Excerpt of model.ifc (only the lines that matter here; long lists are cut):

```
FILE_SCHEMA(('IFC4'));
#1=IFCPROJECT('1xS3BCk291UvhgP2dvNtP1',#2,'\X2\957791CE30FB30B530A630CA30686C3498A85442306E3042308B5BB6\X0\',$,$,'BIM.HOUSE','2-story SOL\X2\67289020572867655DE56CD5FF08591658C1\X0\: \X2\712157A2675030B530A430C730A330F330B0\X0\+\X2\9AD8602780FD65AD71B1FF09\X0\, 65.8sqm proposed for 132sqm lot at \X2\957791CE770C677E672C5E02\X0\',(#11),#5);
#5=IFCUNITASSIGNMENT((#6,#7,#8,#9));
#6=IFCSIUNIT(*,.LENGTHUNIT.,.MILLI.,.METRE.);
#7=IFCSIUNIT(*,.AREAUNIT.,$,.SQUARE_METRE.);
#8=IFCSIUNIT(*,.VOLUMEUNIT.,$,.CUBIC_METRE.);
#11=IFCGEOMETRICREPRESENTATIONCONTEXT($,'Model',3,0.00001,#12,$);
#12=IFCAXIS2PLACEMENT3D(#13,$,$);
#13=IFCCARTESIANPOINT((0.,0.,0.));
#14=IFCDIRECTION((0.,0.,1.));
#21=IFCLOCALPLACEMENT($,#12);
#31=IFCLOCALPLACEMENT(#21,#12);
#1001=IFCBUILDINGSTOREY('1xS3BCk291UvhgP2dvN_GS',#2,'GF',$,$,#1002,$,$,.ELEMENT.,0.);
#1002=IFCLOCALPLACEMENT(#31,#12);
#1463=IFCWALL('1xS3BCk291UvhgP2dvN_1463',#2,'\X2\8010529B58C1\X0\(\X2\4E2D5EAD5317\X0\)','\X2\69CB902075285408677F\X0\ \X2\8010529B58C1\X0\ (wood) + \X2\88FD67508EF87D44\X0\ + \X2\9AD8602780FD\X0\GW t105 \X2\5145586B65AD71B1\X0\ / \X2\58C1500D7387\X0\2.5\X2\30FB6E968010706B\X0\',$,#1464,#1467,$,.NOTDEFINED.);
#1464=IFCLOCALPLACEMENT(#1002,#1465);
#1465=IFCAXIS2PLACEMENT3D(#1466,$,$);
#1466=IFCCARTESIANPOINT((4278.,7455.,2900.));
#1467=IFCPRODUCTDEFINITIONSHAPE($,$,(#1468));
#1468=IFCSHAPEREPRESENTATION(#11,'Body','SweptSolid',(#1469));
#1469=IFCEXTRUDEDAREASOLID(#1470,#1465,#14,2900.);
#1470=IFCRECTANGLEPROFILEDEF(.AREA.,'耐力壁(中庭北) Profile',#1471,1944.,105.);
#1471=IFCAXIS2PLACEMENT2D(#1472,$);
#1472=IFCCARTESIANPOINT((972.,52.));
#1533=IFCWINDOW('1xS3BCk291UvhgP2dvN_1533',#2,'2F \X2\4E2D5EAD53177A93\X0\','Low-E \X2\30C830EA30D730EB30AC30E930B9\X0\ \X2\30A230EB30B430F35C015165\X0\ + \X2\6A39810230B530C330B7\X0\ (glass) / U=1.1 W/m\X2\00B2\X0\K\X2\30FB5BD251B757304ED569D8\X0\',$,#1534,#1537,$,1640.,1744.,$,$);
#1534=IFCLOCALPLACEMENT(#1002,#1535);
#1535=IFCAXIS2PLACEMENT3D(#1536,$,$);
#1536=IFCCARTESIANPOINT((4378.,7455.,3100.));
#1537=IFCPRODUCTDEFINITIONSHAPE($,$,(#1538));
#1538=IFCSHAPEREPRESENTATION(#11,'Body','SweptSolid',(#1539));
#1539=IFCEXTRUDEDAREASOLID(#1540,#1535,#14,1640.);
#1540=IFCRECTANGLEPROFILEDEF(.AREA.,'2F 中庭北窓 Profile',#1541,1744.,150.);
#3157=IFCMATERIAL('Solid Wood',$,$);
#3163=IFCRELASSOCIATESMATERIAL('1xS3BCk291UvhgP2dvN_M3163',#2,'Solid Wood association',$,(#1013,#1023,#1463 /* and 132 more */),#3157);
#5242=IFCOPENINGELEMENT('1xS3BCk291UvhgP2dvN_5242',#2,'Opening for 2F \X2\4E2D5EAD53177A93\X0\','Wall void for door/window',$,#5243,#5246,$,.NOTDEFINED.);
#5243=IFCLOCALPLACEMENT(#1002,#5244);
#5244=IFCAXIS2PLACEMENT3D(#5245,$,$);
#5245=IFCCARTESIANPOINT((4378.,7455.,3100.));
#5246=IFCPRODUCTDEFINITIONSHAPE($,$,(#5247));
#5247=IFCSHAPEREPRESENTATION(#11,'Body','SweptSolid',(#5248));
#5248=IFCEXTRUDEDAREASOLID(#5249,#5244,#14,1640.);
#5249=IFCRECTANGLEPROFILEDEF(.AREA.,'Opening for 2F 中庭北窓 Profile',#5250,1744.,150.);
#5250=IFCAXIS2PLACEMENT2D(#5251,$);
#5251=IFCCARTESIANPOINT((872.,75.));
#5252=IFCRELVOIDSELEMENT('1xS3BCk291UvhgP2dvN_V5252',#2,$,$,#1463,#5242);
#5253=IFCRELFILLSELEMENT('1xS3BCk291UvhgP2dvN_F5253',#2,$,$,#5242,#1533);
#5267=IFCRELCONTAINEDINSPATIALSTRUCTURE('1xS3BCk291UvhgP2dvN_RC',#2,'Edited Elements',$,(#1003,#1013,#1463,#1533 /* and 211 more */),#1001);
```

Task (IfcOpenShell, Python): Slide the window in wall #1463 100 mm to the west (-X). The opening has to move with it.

```python
import ifcopenshell
import ifcopenshell.api.geometry
import ifcopenshell.util.placement
import ifcopenshell.util.unit

model = ifcopenshell.open("model.ifc")
unit_scale = ifcopenshell.util.unit.calculate_unit_scale(model)

window = model.by_guid("1xS3BCk291UvhgP2dvN_1533")
opening = window.FillsVoids[0].RelatingOpeningElement
wall = opening.VoidsElements[0].RelatingBuildingElement

wall_matrix = ifcopenshell.util.placement.get_local_placement(wall.ObjectPlacement)
shift = wall_matrix[:3, 0] * -0.1 / unit_scale
before = ifcopenshell.util.placement.get_local_placement(window.ObjectPlacement)[:3, 3].copy()

# The window is not placed relative to its opening, so move both.
for product in (opening, window):
    matrix = ifcopenshell.util.placement.get_local_placement(product.ObjectPlacement)
    matrix[:3, 3] += shift
    ifcopenshell.api.geometry.edit_object_placement(model, product=product, matrix=matrix, is_si=False)

after = ifcopenshell.util.placement.get_local_placement(window.ObjectPlacement)[:3, 3]
print("window moved by", (after - before).round(3) + 0.0)

model.write("model_rev.ifc")
```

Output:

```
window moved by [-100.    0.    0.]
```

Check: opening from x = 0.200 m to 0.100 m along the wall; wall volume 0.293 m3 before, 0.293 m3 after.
